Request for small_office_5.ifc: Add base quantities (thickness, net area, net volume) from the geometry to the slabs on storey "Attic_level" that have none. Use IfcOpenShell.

First a look at what the model holds.

```python
import ifcopenshell
import ifcopenshell.util.element
import ifcopenshell.util.unit

model = ifcopenshell.open("small_office_5.ifc")
print(model.schema)
for unit_type in ("LENGTHUNIT", "AREAUNIT", "VOLUMEUNIT"):
    print(unit_type, ifcopenshell.util.unit.calculate_unit_scale(model, unit_type))
storey = next(s for s in model.by_type("IfcBuildingStorey") if s.Name == "Attic_level")
slabs = [e for e in ifcopenshell.util.element.get_decomposition(storey) if e.is_a("IfcSlab")]
for e in sorted(slabs, key=lambda e: e.id()):
    print(e.id(), e.is_a(), e.Name, list(ifcopenshell.util.element.get_psets(e, qtos_only=True)), sep=" | ")
```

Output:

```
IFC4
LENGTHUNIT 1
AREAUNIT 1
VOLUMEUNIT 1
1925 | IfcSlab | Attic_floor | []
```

```python
import ifcopenshell
import ifcopenshell.api.pset
import ifcopenshell.geom
import ifcopenshell.util.element
import ifcopenshell.util.shape
import ifcopenshell.util.unit

model = ifcopenshell.open("small_office_5.ifc")
unit_scale = ifcopenshell.util.unit.calculate_unit_scale(model)
area_scale = ifcopenshell.util.unit.calculate_unit_scale(model, "AREAUNIT")
volume_scale = ifcopenshell.util.unit.calculate_unit_scale(model, "VOLUMEUNIT")
settings = ifcopenshell.geom.settings()

storey = next(s for s in model.by_type("IfcBuildingStorey") if s.Name == "Attic_level")
slabs = [e for e in ifcopenshell.util.element.get_decomposition(storey) if e.is_a("IfcSlab")]

for e in sorted(slabs, key=lambda e: e.id()):
    if ifcopenshell.util.element.get_psets(e, qtos_only=True, should_inherit=False):
        continue
    # Geometry comes back in metres, in the element's own axes.
    shape = ifcopenshell.geom.create_shape(settings, e)
    values = {
        "Width": ifcopenshell.util.shape.get_z(shape.geometry) / unit_scale,
        "NetArea": ifcopenshell.util.shape.get_footprint_area(shape.geometry) / area_scale,
        "NetVolume": ifcopenshell.util.shape.get_volume(shape.geometry) / volume_scale,
    }
    qto = ifcopenshell.api.pset.add_qto(model, product=e, name="Qto_SlabBaseQuantities")
    ifcopenshell.api.pset.edit_qto(model, qto=qto, properties=values)
    print(e.id(), {k: round(v, 3) for k, v in values.items()})

model.write("small_office_5_edited.ifc")
```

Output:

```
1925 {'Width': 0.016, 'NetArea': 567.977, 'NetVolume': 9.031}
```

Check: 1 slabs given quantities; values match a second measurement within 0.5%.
